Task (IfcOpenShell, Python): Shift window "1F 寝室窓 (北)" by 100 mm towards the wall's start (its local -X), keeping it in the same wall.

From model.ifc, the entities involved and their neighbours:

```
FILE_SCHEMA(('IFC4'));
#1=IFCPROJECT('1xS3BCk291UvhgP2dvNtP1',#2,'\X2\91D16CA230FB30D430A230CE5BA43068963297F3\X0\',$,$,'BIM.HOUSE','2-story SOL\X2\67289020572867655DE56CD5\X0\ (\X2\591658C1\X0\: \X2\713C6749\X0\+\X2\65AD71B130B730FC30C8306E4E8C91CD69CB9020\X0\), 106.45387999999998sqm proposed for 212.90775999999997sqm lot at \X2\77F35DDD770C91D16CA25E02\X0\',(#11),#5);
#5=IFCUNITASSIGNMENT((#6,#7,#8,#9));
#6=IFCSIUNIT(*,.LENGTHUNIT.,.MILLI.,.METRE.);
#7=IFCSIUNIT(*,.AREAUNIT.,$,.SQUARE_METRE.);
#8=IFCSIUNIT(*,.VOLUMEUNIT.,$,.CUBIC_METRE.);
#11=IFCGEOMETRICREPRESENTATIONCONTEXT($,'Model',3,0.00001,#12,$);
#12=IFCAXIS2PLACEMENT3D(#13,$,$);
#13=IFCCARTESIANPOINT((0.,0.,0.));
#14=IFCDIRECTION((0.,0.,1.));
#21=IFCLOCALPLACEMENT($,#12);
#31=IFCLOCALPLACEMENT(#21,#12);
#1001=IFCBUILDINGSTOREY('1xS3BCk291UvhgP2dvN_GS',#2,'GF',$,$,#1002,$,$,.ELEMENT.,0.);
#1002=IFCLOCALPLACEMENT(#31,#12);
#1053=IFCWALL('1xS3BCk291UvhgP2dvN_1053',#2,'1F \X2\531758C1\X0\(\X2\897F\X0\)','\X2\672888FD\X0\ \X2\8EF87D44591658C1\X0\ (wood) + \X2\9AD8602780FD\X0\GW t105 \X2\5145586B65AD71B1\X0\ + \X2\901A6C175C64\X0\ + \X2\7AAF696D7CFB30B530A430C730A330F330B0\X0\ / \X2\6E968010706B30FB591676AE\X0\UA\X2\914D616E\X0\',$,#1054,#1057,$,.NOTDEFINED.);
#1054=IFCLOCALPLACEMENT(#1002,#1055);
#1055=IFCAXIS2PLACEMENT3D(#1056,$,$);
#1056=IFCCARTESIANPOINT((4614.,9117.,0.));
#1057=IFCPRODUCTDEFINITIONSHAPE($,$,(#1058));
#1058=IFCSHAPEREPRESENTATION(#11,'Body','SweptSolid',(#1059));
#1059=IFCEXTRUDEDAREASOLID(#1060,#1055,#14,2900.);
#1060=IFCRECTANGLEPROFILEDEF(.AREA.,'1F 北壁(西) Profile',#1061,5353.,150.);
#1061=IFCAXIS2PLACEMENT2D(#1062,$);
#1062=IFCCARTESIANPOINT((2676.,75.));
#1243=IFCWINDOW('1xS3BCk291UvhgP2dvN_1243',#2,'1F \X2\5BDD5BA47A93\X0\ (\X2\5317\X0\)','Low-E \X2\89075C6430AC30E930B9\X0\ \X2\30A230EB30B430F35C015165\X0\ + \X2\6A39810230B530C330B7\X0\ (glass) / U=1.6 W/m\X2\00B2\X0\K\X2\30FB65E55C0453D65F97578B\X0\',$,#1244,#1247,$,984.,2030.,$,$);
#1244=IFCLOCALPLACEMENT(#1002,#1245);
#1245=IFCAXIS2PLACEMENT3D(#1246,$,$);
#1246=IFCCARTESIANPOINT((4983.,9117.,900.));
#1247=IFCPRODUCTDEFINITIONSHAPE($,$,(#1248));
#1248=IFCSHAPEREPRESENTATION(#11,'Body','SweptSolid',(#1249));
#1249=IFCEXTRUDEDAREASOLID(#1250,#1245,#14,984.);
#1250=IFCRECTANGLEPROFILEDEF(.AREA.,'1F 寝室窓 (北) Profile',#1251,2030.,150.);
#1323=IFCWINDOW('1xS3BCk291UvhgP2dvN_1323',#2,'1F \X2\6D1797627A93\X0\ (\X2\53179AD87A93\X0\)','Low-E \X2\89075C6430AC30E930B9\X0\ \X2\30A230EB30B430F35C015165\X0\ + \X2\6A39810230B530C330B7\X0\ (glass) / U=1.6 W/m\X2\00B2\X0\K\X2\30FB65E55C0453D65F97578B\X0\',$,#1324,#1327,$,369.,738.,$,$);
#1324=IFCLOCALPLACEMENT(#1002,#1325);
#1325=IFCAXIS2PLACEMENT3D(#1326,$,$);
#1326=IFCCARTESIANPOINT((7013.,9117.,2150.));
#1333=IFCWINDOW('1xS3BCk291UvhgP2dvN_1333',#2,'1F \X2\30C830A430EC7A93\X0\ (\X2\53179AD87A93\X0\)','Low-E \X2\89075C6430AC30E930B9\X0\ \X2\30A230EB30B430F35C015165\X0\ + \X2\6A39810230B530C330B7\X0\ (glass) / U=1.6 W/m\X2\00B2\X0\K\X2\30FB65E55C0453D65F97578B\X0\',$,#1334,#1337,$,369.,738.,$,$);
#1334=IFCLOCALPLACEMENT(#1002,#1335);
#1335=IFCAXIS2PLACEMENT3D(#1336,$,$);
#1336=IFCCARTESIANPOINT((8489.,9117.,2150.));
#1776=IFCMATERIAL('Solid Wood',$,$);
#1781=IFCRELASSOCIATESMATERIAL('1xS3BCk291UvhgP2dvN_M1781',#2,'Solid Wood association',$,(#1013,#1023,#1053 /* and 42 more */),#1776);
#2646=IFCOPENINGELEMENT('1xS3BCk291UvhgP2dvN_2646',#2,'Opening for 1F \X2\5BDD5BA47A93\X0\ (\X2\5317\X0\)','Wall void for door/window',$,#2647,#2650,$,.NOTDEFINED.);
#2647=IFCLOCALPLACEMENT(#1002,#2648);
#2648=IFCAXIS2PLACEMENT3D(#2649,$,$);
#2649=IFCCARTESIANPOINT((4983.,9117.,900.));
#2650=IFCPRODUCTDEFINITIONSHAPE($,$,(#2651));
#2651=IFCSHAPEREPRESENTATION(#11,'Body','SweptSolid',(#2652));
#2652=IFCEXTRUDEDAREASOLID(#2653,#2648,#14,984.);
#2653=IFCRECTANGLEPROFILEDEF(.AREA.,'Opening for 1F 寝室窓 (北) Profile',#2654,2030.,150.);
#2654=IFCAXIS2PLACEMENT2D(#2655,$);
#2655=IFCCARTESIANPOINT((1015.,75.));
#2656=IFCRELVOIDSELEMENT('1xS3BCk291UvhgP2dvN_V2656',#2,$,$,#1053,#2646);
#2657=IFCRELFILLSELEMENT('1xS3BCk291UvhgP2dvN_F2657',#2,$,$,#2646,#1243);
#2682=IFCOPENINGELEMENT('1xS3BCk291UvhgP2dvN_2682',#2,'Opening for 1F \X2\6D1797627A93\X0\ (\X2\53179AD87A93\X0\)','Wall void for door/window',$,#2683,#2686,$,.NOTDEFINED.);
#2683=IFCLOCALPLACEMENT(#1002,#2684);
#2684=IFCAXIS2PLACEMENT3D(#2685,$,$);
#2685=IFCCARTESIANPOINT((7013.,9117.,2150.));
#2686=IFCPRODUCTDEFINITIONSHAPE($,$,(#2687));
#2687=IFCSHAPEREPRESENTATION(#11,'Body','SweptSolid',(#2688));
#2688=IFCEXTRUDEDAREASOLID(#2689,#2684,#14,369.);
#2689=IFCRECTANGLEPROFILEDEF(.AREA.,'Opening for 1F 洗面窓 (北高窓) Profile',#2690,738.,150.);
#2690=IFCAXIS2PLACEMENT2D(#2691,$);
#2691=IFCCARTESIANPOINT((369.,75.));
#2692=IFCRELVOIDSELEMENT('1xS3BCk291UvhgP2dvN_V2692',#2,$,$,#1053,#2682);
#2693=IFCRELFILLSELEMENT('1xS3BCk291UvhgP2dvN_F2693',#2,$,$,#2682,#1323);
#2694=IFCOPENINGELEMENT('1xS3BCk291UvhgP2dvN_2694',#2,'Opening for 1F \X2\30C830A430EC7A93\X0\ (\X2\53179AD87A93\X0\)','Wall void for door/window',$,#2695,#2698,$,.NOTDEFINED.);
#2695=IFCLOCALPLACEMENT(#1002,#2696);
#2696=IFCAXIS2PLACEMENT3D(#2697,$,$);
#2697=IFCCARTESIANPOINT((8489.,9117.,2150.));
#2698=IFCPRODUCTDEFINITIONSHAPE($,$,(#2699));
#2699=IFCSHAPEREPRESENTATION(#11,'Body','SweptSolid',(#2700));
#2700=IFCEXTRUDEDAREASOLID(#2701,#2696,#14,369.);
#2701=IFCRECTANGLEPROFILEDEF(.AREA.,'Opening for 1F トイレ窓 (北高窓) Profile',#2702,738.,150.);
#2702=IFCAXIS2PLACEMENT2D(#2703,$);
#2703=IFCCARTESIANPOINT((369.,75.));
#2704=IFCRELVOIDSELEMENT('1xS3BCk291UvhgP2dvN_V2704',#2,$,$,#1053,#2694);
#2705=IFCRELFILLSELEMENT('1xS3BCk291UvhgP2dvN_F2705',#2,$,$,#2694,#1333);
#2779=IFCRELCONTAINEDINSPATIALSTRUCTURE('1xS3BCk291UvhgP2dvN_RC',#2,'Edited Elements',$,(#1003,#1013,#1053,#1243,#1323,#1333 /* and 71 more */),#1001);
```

```python
import ifcopenshell
import ifcopenshell.api.geometry
import ifcopenshell.util.placement

model = ifcopenshell.open("model.ifc")

window = model.by_guid("1xS3BCk291UvhgP2dvN_1243")
opening = window.FillsVoids[0].RelatingOpeningElement
wall = opening.VoidsElements[0].RelatingBuildingElement

wall_matrix = ifcopenshell.util.placement.get_local_placement(wall.ObjectPlacement)
shift = wall_matrix[:3, 0] * -100.0
before = ifcopenshell.util.placement.get_local_placement(window.ObjectPlacement)[:3, 3].copy()

# The window is not placed relative to its opening, so move both.
for product in (opening, window):
    matrix = ifcopenshell.util.placement.get_local_placement(product.ObjectPlacement)
    matrix[:3, 3] += shift
    ifcopenshell.api.geometry.edit_object_placement(model, product=product, matrix=matrix, is_si=False)

after = ifcopenshell.util.placement.get_local_placement(window.ObjectPlacement)[:3, 3]
print("window moved by", (after - before).round(3) + 0.0)

model.write("model_updated.ifc")
```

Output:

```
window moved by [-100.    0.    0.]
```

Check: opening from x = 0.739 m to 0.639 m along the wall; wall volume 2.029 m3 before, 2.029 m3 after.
